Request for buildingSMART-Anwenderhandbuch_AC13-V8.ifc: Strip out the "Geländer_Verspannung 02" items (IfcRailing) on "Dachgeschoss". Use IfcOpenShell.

First a look at what the model holds.

```python
import ifcopenshell
import ifcopenshell.util.element

model = ifcopenshell.open("buildingSMART-Anwenderhandbuch_AC13-V8.ifc")
print(model.schema)
storey = next(s for s in model.by_type("IfcBuildingStorey") if s.Name == "Dachgeschoss")
railings = [e for e in ifcopenshell.util.element.get_decomposition(storey) if e.is_a("IfcRailing")]
seen = {}
for e in railings:
    element_type = ifcopenshell.util.element.get_type(e)
    name = element_type.Name if element_type not in (None, e) else None
    seen[name] = seen.get(name, 0) + 1
for name, count in sorted(seen.items(), key=str):
    print(count, "x", name)
```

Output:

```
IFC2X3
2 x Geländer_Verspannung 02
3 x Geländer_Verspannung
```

```python
import ifcopenshell
import ifcopenshell.api.root
import ifcopenshell.util.element

model = ifcopenshell.open("buildingSMART-Anwenderhandbuch_AC13-V8.ifc")

storey = next(s for s in model.by_type("IfcBuildingStorey") if s.Name == "Dachgeschoss")
railings = [e for e in ifcopenshell.util.element.get_decomposition(storey) if e.is_a("IfcRailing")]
targets = [e for e in railings if (t := ifcopenshell.util.element.get_type(e)) not in (None, e) and t.Name == "Geländer_Verspannung 02"]

for e in targets:
    ifcopenshell.api.root.remove_product(model, product=e)
print(len(targets), "removed")

model.write("buildingSMART-Anwenderhandbuch_AC13-V8_v2.ifc")
```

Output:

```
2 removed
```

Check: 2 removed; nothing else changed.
